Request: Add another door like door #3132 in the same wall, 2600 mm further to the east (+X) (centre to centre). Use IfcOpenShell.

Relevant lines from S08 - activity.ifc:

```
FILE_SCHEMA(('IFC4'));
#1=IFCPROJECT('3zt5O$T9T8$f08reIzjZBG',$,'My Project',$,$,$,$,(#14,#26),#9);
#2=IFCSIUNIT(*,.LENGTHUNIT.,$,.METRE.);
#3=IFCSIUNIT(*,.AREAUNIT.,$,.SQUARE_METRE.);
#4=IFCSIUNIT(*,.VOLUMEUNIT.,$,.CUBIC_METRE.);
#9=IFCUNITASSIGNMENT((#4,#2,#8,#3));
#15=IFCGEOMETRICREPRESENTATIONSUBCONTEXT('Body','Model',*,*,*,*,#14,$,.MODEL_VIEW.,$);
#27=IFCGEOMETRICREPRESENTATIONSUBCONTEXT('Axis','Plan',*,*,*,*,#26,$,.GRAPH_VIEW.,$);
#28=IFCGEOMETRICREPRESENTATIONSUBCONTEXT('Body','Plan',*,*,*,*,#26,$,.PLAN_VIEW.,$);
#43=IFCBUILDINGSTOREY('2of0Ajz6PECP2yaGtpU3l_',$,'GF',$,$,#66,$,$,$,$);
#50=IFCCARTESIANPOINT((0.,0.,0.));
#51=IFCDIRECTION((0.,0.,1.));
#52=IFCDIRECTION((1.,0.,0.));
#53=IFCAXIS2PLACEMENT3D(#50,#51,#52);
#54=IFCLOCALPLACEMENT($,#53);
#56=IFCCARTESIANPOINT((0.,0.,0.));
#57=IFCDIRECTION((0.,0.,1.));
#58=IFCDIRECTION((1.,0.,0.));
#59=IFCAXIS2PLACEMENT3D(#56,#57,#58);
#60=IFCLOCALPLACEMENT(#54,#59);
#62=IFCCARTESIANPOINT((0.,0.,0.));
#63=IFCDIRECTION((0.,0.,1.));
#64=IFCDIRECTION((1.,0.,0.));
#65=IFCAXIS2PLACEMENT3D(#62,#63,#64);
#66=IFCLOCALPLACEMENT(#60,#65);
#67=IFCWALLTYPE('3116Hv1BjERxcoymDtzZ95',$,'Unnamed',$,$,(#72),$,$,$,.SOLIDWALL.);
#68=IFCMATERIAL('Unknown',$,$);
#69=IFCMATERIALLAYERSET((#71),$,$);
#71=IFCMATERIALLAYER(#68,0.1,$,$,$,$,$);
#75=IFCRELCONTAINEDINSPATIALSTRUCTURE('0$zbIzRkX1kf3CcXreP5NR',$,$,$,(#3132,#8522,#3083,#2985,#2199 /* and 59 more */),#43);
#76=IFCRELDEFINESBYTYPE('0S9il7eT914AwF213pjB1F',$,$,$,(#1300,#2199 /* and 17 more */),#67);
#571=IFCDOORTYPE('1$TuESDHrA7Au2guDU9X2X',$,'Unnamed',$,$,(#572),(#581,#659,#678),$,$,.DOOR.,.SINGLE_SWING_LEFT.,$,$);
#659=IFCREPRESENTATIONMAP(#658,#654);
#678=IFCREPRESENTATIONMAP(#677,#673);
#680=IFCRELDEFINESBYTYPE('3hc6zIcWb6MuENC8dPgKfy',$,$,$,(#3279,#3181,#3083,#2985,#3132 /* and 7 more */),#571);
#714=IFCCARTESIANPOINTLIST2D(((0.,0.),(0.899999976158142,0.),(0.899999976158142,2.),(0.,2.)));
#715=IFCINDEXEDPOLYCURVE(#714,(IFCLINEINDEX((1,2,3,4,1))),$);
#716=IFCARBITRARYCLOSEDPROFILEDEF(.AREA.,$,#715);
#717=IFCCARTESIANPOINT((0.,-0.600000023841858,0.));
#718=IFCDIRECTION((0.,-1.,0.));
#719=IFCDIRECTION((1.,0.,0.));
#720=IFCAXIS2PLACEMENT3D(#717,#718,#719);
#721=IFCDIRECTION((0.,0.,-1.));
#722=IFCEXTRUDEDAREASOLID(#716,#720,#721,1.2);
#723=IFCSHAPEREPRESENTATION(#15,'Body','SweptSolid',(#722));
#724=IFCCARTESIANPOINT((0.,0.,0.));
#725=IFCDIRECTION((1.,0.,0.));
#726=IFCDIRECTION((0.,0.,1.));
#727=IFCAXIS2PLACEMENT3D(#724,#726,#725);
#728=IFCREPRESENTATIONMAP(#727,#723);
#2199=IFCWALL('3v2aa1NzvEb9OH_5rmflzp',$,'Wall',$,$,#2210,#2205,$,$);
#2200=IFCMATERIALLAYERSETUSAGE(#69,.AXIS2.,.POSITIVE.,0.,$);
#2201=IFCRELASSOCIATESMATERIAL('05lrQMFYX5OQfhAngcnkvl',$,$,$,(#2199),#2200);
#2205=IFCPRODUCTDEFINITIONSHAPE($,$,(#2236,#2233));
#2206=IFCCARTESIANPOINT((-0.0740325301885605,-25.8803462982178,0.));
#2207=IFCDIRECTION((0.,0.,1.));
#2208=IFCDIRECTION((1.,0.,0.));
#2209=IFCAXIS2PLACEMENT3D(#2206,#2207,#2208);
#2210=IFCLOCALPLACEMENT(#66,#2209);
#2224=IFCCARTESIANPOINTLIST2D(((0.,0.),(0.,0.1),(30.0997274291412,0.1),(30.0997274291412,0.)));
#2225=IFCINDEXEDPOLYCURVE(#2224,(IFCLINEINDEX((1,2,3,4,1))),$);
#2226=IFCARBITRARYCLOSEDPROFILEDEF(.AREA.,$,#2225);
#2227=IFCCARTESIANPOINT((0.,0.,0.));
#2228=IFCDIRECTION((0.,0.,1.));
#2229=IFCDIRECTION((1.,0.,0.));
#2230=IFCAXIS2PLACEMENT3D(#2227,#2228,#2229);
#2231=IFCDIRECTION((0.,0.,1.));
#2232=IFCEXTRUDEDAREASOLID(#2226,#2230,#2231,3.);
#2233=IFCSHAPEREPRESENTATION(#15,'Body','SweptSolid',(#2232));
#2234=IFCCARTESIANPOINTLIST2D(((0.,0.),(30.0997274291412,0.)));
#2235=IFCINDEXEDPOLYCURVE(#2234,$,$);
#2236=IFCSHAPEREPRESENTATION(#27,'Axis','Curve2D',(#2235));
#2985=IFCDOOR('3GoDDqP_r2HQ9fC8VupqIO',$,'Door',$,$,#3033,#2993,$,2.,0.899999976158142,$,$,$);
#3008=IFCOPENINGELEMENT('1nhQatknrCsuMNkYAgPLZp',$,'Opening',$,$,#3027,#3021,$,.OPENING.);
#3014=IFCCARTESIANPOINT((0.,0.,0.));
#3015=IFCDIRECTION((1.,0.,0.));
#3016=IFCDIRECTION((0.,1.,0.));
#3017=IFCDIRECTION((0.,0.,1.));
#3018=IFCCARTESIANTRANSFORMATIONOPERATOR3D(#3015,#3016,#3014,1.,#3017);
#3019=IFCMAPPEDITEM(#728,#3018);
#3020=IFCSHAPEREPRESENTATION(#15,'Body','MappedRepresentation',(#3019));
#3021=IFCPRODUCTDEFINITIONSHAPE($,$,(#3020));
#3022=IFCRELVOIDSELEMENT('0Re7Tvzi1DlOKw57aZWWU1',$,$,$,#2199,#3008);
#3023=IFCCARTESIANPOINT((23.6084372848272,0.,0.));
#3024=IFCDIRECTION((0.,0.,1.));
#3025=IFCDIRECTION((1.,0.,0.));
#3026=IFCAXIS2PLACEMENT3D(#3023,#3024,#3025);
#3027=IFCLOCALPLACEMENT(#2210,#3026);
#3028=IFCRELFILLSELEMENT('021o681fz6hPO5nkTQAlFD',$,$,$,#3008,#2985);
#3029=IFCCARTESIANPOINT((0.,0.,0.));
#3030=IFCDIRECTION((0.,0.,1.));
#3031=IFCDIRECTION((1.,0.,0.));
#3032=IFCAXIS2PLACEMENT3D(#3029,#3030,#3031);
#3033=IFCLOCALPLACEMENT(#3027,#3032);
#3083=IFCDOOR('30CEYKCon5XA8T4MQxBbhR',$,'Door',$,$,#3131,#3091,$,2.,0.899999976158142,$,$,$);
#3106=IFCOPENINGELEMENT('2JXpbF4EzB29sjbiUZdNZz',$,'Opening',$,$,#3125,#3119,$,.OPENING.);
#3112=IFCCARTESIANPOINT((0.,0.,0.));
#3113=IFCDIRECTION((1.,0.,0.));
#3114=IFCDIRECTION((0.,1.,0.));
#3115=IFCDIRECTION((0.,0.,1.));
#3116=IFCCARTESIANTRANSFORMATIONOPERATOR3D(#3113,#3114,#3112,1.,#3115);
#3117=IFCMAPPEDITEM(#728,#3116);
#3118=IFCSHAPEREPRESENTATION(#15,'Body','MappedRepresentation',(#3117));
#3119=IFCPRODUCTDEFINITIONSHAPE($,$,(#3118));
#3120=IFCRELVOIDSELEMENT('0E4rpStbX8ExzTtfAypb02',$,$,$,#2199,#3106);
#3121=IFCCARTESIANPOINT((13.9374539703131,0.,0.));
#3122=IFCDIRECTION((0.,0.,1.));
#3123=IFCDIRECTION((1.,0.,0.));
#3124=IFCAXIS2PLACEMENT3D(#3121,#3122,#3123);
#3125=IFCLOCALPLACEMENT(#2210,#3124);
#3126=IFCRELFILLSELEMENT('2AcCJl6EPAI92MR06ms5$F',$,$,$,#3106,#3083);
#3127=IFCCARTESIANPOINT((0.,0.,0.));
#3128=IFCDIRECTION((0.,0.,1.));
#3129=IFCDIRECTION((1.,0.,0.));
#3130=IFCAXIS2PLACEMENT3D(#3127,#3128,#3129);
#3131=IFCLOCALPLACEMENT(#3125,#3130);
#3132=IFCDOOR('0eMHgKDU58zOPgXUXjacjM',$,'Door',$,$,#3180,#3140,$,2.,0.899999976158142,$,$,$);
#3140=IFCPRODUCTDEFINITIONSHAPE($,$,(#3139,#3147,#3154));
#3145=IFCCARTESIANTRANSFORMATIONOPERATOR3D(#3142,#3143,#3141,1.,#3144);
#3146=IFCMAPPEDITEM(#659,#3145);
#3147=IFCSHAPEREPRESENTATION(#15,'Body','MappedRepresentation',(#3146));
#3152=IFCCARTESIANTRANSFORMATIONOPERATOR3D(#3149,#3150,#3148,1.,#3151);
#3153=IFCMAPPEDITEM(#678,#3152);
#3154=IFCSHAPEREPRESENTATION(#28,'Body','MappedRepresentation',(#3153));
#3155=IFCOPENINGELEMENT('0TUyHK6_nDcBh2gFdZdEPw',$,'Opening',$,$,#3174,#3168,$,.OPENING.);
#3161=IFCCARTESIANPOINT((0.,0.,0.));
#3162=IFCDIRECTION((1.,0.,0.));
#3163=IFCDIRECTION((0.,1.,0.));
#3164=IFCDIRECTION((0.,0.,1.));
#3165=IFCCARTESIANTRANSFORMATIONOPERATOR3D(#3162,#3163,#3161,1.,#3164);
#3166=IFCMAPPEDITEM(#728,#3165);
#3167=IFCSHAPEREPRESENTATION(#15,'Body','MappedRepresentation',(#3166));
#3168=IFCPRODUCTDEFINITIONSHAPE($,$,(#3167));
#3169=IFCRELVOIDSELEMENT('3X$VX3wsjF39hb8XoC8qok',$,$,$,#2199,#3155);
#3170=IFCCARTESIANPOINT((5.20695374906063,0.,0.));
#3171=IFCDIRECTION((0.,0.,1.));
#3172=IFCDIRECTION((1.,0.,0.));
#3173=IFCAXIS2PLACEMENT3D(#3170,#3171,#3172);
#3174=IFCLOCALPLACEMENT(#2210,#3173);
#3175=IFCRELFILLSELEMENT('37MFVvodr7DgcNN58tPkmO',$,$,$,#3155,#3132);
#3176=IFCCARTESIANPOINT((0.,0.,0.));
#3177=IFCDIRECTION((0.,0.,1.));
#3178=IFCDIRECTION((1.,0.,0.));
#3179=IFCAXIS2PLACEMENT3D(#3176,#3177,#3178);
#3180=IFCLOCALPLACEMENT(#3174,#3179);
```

```python
import ifcopenshell
import ifcopenshell.api.feature
import ifcopenshell.api.geometry
import ifcopenshell.api.root
import ifcopenshell.geom
import ifcopenshell.util.element
import ifcopenshell.util.placement
import ifcopenshell.util.shape

model = ifcopenshell.open("S08 - activity.ifc")
settings = ifcopenshell.geom.settings()


def volume(element):
    """Net volume in cubic metres, openings subtracted."""
    shape = ifcopenshell.geom.create_shape(settings, element)
    return ifcopenshell.util.shape.get_volume(shape.geometry)


door = model.by_guid("0eMHgKDU58zOPgXUXjacjM")
opening = door.FillsVoids[0].RelatingOpeningElement
wall = opening.VoidsElements[0].RelatingBuildingElement
before = volume(wall)
shift = ifcopenshell.util.placement.get_local_placement(wall.ObjectPlacement)[:3, 0] * 2.6

# copy_class copies the void relationship, type, container and properties, but no geometry.
new_opening = ifcopenshell.api.root.copy_class(model, product=opening)
new_opening.Representation = ifcopenshell.util.element.copy_deep(
    model, opening.Representation, exclude=["IfcGeometricRepresentationContext", "IfcRepresentationMap"]
)
new_door = ifcopenshell.api.root.copy_class(model, product=door)
new_door.Representation = ifcopenshell.util.element.copy_deep(
    model, door.Representation, exclude=["IfcGeometricRepresentationContext", "IfcRepresentationMap"]
)
ifcopenshell.api.feature.add_filling(model, opening=new_opening, element=new_door)

for old, new in ((opening, new_opening), (door, new_door)):
    matrix = ifcopenshell.util.placement.get_local_placement(old.ObjectPlacement)
    matrix[:3, 3] += shift
    ifcopenshell.api.geometry.edit_object_placement(model, product=new, matrix=matrix, is_si=False)

after = volume(wall)

print(f"wall volume {before:.3f} -> {after:.3f} m3")

model.write("S08 - activity_updated.ifc")
```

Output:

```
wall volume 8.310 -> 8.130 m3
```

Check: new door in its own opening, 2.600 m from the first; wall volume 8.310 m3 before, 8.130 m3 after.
